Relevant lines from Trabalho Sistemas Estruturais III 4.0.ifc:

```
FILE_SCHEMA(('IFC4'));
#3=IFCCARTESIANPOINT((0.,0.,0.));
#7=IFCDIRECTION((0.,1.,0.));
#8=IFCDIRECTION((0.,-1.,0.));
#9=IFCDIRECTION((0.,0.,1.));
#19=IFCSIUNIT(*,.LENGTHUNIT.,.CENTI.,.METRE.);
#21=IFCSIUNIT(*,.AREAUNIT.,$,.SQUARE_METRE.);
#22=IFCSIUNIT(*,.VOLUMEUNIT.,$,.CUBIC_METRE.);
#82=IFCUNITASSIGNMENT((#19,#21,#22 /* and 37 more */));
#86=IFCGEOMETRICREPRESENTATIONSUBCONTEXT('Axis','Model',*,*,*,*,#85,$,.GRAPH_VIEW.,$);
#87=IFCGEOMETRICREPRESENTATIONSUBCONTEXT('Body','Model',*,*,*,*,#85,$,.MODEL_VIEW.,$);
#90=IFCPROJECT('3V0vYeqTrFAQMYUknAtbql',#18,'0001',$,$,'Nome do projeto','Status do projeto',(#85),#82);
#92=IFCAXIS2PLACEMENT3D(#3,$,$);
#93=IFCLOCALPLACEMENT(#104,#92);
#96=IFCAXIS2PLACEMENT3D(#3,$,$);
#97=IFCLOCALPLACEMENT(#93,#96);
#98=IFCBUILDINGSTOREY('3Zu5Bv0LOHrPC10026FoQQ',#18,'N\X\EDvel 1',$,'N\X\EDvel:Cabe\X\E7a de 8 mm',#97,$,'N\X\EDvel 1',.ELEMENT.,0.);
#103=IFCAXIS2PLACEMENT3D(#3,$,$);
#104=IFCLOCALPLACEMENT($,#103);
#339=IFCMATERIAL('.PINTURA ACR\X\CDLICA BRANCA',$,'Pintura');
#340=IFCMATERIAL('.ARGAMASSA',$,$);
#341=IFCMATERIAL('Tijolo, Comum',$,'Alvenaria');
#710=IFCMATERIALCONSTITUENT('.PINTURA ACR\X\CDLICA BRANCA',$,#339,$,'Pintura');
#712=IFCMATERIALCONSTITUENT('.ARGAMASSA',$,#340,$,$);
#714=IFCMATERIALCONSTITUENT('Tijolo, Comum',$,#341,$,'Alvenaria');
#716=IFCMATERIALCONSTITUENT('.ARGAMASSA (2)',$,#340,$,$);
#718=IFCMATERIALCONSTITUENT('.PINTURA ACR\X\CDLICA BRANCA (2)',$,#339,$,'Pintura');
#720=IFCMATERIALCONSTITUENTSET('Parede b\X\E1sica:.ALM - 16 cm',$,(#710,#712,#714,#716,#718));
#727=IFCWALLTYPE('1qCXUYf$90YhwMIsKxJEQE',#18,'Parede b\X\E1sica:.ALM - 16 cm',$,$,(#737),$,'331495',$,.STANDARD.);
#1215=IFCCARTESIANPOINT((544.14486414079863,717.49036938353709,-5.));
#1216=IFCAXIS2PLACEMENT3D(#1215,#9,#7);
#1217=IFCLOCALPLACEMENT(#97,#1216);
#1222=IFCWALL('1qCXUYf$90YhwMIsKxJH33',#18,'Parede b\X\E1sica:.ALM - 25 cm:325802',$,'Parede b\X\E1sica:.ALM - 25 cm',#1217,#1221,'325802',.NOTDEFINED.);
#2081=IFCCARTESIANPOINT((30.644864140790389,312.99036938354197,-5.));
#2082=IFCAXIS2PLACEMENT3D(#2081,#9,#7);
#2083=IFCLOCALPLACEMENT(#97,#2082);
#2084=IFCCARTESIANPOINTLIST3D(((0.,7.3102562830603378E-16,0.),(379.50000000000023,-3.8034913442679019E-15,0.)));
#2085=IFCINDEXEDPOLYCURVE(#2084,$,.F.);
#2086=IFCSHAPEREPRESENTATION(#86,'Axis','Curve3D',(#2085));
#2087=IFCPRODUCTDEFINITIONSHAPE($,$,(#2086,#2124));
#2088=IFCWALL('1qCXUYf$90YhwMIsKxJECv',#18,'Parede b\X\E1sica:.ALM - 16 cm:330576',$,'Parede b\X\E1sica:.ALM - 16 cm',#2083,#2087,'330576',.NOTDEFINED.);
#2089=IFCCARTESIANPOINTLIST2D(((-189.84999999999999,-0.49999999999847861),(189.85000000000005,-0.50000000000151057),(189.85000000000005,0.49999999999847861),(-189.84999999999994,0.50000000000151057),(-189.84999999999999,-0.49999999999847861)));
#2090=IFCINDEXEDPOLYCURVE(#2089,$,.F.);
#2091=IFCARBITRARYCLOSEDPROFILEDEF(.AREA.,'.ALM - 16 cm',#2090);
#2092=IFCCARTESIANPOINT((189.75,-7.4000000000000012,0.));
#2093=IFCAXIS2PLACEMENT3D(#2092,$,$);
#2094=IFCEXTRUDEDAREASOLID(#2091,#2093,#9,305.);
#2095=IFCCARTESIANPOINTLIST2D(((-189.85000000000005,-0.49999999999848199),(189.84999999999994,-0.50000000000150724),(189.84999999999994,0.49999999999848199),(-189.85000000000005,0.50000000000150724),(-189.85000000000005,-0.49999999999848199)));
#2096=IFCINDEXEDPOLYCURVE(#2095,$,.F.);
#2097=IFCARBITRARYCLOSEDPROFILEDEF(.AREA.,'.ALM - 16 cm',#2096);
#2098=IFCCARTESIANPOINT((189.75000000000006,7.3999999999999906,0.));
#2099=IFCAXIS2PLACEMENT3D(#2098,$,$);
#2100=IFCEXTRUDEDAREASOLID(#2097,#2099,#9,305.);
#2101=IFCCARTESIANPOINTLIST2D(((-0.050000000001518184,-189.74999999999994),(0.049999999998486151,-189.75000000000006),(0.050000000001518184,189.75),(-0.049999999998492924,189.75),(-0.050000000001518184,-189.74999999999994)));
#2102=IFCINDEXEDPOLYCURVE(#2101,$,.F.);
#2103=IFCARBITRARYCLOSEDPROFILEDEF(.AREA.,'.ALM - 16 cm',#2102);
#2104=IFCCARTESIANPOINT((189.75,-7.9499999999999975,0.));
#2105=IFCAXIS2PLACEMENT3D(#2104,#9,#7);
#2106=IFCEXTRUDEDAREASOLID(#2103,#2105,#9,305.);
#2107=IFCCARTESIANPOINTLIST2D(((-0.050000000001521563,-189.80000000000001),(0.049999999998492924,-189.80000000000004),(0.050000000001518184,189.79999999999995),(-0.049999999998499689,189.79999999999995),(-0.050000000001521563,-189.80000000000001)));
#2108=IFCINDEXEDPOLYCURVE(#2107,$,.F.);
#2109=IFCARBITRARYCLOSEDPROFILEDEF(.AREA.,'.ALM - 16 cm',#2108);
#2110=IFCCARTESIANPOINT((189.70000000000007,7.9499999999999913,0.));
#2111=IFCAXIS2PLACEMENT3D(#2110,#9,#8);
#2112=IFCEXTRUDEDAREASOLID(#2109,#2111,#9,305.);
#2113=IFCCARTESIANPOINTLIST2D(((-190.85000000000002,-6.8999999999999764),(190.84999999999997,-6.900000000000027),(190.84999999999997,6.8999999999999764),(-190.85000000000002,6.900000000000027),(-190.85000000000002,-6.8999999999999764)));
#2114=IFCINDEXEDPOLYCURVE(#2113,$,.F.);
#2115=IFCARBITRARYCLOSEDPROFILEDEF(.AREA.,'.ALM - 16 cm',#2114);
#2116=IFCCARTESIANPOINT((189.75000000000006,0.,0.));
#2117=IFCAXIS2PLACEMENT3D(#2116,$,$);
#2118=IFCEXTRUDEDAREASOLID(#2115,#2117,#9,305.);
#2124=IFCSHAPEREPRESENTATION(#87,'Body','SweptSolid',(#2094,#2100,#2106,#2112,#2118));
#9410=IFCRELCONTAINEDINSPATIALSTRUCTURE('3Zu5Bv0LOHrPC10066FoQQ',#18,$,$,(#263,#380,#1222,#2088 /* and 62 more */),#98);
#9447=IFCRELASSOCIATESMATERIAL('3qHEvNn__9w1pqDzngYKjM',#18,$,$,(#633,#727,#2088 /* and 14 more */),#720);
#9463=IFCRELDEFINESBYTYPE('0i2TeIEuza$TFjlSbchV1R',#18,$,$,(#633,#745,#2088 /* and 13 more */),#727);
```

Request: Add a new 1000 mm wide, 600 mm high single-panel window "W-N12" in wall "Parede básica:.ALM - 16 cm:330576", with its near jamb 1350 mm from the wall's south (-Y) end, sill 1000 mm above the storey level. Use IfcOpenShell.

```python
import numpy as np
import ifcopenshell
import ifcopenshell.api.feature
import ifcopenshell.api.geometry
import ifcopenshell.api.root
import ifcopenshell.api.spatial
import ifcopenshell.geom
import ifcopenshell.util.element
import ifcopenshell.util.placement
import ifcopenshell.util.representation
import ifcopenshell.util.shape
import ifcopenshell.util.unit

model = ifcopenshell.open("Trabalho Sistemas Estruturais III 4.0.ifc")
unit_scale = ifcopenshell.util.unit.calculate_unit_scale(model)
settings = ifcopenshell.geom.settings()


def volume(element):
    """Net volume in cubic metres, openings subtracted."""
    shape = ifcopenshell.geom.create_shape(settings, element)
    return ifcopenshell.util.shape.get_volume(shape.geometry)


wall = model.by_id(2088)
storey = ifcopenshell.util.element.get_container(wall, ifc_class="IfcBuildingStorey")
context = ifcopenshell.util.representation.get_context(model, "Model", "Body", "MODEL_VIEW")
before = volume(wall)

width, height, from_end, sill = 1, 0.6, 1.35, 1  # metres

# The wall runs along its own X axis, and the end named is its -X end.
wall_shape = ifcopenshell.geom.create_shape(settings, wall)
x, y, z = ifcopenshell.util.shape.get_vertices(wall_shape.geometry).T
start = x.min() + from_end
face, thickness = float(y.min()), float(y.max() - y.min())
wall_matrix = ifcopenshell.util.placement.get_local_placement(wall.ObjectPlacement)
level = ifcopenshell.util.placement.get_local_placement(storey.ObjectPlacement)[2, 3]


def in_wall(x, y):
    """Placement at x, y metres in the wall's axes, at sill height."""
    matrix = wall_matrix.copy()
    matrix[:, 3] = wall_matrix @ np.array([x / unit_scale, y / unit_scale, 0.0, 1.0])
    matrix[2, 3] = level + sill / unit_scale
    return matrix


# Opening: a box that overshoots both wall faces by 50 mm.
opening = ifcopenshell.api.root.create_entity(model, ifc_class="IfcOpeningElement", predefined_type="OPENING")
box = ifcopenshell.api.geometry.add_wall_representation(
    model, context=context, length=width, height=height, thickness=thickness + 0.1
)
ifcopenshell.api.geometry.assign_representation(model, product=opening, representation=box)
ifcopenshell.api.geometry.edit_object_placement(model, product=opening, matrix=in_wall(start, face - 0.05), is_si=False)
ifcopenshell.api.feature.add_feature(model, feature=opening, element=wall)

window = ifcopenshell.api.root.create_entity(model, ifc_class="IfcWindow", name="W-N12", predefined_type="WINDOW")
window.OverallWidth, window.OverallHeight = width / unit_scale, height / unit_scale
window.PartitioningType = "SINGLE_PANEL"
body = ifcopenshell.api.geometry.add_window_representation(
    model,
    context=context,
    overall_width=window.OverallWidth,
    overall_height=window.OverallHeight,
    partition_type="SINGLE_PANEL",
)
ifcopenshell.api.geometry.assign_representation(model, product=window, representation=body)
ifcopenshell.api.spatial.assign_container(model, products=[window], relating_structure=storey)
ifcopenshell.api.feature.add_filling(model, opening=opening, element=window)

# Centre the window in the wall's thickness.
ifcopenshell.api.geometry.edit_object_placement(model, product=window, matrix=in_wall(start, face), is_si=False)
window_shape = ifcopenshell.geom.create_shape(settings, window)
depth = ifcopenshell.util.shape.get_vertices(window_shape.geometry)[:, 1]
offset = face + thickness / 2 - (depth.min() + depth.max()) / 2
ifcopenshell.api.geometry.edit_object_placement(model, product=window, matrix=in_wall(start, offset), is_si=False)

after = volume(wall)

print(f"wall volume {before:.3f} -> {after:.3f} m3")

model.write("Trabalho Sistemas Estruturais III 4.0_edited.ifc")
```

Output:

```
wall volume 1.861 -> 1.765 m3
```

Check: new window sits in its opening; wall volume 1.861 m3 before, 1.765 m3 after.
